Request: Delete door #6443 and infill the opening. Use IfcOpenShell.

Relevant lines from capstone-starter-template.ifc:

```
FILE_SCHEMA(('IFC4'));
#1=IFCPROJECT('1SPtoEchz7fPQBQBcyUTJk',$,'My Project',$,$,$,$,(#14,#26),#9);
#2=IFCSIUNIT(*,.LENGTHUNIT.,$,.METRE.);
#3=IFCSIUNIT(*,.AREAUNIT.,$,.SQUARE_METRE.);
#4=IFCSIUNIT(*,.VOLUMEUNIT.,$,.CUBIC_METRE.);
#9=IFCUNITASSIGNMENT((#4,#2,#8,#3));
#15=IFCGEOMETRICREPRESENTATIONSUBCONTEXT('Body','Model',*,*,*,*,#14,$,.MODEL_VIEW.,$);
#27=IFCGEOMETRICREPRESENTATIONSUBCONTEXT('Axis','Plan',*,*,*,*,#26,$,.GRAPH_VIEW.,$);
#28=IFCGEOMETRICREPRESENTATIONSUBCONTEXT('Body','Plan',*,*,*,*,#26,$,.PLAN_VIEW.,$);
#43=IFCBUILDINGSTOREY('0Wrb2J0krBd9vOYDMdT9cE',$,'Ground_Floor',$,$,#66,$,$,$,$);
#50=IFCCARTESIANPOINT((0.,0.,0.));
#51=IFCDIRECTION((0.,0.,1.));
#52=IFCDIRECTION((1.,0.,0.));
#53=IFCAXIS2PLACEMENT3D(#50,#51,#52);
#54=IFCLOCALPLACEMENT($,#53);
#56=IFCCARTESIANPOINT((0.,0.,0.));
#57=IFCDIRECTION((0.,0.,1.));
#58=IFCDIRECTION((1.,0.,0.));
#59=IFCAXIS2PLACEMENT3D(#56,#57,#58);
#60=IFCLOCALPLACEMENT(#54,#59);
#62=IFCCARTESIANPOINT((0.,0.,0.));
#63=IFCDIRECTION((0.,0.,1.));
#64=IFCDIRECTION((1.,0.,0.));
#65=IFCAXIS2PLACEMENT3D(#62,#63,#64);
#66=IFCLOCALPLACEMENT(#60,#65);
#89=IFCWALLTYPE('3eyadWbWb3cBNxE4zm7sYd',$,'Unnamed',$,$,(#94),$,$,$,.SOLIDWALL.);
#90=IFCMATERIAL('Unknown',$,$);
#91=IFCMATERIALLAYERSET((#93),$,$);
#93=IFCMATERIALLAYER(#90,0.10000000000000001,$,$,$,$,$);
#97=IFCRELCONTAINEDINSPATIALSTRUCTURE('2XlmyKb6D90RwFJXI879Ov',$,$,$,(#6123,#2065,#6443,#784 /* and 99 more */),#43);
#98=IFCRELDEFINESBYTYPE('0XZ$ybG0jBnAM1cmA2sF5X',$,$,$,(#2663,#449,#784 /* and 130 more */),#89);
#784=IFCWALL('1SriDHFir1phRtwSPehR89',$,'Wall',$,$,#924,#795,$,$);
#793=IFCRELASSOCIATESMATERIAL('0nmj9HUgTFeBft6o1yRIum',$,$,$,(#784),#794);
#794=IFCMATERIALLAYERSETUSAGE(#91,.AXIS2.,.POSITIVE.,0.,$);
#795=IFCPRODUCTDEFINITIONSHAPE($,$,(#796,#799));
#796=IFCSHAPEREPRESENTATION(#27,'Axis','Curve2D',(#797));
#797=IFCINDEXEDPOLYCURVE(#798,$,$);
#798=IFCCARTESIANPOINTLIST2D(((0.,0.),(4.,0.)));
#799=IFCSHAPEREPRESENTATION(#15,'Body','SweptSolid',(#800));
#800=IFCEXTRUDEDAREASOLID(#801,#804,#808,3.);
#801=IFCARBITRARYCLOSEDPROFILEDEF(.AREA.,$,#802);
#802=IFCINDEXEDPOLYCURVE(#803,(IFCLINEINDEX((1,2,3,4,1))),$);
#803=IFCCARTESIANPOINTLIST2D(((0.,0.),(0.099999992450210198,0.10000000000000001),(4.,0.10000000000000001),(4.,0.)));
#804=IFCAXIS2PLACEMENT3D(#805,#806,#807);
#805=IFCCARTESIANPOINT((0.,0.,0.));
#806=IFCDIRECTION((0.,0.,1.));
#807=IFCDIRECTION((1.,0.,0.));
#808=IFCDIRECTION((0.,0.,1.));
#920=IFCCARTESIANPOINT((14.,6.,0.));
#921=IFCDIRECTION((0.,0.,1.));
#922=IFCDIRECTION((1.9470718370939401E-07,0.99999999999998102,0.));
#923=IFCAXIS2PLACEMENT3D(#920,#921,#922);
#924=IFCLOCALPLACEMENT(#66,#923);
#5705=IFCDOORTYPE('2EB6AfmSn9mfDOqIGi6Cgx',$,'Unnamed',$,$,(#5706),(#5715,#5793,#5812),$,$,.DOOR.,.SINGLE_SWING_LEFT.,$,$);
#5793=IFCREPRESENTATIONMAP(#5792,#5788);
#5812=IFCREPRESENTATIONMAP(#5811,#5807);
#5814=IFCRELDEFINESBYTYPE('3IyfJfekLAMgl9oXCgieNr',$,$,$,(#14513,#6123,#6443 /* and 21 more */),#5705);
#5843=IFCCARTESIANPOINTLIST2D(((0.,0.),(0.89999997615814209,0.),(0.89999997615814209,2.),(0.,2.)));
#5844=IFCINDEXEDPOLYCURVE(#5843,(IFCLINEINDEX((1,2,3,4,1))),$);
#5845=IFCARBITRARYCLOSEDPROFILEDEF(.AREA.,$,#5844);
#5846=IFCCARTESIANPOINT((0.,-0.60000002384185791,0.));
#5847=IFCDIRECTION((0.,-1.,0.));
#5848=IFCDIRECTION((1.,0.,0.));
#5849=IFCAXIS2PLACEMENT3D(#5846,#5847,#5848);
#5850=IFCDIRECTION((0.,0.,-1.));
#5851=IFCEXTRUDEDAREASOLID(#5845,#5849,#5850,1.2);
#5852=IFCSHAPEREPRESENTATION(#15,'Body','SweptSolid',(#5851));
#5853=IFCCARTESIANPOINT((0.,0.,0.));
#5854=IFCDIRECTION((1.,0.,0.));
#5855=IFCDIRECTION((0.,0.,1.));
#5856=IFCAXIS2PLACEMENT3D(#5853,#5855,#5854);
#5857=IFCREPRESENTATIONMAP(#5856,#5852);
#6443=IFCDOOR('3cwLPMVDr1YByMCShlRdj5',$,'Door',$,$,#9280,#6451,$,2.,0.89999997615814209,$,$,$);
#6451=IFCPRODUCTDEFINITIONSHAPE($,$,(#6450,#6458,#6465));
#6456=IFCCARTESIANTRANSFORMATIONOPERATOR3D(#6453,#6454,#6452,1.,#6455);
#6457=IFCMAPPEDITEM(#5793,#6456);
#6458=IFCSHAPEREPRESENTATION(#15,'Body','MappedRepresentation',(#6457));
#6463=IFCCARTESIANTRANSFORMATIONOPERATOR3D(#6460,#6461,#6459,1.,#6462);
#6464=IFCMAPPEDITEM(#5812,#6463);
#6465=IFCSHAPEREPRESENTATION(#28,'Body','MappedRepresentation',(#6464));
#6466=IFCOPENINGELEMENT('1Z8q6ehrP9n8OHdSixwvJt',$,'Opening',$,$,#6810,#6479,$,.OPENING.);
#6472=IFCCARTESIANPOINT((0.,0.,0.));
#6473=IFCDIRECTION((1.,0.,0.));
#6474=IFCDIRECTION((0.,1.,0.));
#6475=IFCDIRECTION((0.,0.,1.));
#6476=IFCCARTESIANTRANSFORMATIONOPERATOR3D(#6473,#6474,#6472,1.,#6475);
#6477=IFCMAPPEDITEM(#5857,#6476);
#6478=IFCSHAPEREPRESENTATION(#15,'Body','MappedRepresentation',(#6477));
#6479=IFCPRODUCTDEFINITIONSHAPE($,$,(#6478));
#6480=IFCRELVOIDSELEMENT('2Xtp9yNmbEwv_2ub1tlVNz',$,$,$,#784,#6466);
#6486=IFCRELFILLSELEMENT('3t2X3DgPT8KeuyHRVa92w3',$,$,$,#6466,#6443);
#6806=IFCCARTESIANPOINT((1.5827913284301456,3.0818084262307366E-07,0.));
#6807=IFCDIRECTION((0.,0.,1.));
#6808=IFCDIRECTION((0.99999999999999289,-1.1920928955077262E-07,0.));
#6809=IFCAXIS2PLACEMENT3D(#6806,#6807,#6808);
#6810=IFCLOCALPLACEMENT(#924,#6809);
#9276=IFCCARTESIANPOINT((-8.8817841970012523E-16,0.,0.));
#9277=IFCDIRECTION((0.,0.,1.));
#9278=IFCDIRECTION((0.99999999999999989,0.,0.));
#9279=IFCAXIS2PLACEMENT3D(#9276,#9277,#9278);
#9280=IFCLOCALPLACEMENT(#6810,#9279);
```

```python
import ifcopenshell
import ifcopenshell.api.feature
import ifcopenshell.api.root
import ifcopenshell.geom
import ifcopenshell.util.shape

model = ifcopenshell.open("capstone-starter-template.ifc")
settings = ifcopenshell.geom.settings()


def volume(element):
    """Net volume in cubic metres, openings subtracted."""
    shape = ifcopenshell.geom.create_shape(settings, element)
    return ifcopenshell.util.shape.get_volume(shape.geometry)


door = model.by_guid("3cwLPMVDr1YByMCShlRdj5")
opening = door.FillsVoids[0].RelatingOpeningElement
wall = opening.VoidsElements[0].RelatingBuildingElement
before = volume(wall)

ifcopenshell.api.root.remove_product(model, product=door)
ifcopenshell.api.feature.remove_feature(model, feature=opening)

after = volume(wall)

print(f"wall volume {before:.3f} -> {after:.3f} m3")

model.write("capstone-starter-template_updated.ifc")
```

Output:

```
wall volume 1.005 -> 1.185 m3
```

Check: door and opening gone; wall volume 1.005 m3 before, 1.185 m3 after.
